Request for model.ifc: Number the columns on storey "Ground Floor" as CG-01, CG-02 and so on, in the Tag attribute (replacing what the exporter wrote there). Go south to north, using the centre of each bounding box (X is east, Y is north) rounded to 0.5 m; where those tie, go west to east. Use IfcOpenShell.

First a look at what the model holds.

```python
import ifcopenshell
import ifcopenshell.util.element
import ifcopenshell.util.placement

model = ifcopenshell.open("model.ifc")
print(model.schema)
storey = next(s for s in model.by_type("IfcBuildingStorey") if s.Name == "Ground Floor")
columns = [e for e in ifcopenshell.util.element.get_decomposition(storey) if e.is_a("IfcColumn")]
for e in sorted(columns, key=lambda e: e.id()):
    origin = ifcopenshell.util.placement.get_local_placement(e.ObjectPlacement)[:3, 3]
    print(e.id(), e.Tag, e.Name, origin.round(2) + 0.0, sep=" | ")
```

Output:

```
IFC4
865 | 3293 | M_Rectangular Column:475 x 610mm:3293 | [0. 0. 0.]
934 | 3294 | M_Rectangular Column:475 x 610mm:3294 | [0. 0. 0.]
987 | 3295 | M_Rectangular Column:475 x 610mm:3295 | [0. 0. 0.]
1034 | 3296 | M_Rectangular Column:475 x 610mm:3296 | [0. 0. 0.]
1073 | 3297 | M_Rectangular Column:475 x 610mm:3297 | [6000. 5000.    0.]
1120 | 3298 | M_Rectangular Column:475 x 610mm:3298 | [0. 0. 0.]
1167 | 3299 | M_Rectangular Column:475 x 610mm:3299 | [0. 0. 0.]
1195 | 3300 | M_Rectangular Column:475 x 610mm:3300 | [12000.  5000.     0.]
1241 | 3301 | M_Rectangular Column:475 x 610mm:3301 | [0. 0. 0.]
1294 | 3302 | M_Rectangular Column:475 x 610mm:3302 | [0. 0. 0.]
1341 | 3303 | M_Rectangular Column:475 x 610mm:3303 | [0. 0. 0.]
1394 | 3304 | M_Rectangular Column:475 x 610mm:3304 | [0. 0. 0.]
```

```python
import ifcopenshell
import ifcopenshell.geom
import ifcopenshell.util.element
import ifcopenshell.util.shape

model = ifcopenshell.open("model.ifc")
settings = ifcopenshell.geom.settings()
settings.set("use-world-coords", True)


def centre(element):
    shape = ifcopenshell.geom.create_shape(settings, element)
    return ifcopenshell.util.shape.get_bbox_centroid(shape.geometry)


storey = next(s for s in model.by_type("IfcBuildingStorey") if s.Name == "Ground Floor")
columns = [e for e in ifcopenshell.util.element.get_decomposition(storey) if e.is_a("IfcColumn")]

# Insertion points can sit at a corner or the storey origin, so sort by the geometry (in metres).
centres = {e: centre(e) for e in columns}
columns.sort(key=lambda e: (round(centres[e][1] / 0.5), centres[e][0]))

for i, e in enumerate(columns, start=1):
    number = f"CG-{i:02d}"
    e.Tag = number
    print(e.id(), number)

model.write("model-out.ifc")
```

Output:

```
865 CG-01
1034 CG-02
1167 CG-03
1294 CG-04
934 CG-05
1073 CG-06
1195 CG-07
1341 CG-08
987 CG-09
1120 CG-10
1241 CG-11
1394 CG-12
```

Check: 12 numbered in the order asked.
